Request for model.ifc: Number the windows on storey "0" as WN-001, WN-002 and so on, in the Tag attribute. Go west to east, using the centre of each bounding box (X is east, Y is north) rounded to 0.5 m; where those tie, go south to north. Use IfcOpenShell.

First a look at what the model holds.

```python
import ifcopenshell
import ifcopenshell.util.element
import ifcopenshell.util.placement

model = ifcopenshell.open("model.ifc")
print(model.schema)
storey = next(s for s in model.by_type("IfcBuildingStorey") if s.Name == "0")
windows = [e for e in ifcopenshell.util.element.get_decomposition(storey) if e.is_a("IfcWindow")]
for e in sorted(windows, key=lambda e: e.id()):
    origin = ifcopenshell.util.placement.get_local_placement(e.ObjectPlacement)[:3, 3]
    print(e.id(), e.Tag, e.Name, origin.round(2) + 0.0, sep=" | ")
```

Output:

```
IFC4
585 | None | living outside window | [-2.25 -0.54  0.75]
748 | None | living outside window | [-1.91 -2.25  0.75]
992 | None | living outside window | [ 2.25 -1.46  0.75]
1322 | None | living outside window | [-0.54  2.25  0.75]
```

```python
import ifcopenshell
import ifcopenshell.geom
import ifcopenshell.util.element
import ifcopenshell.util.shape

model = ifcopenshell.open("model.ifc")
settings = ifcopenshell.geom.settings()
settings.set("use-world-coords", True)


def centre(element):
    shape = ifcopenshell.geom.create_shape(settings, element)
    return ifcopenshell.util.shape.get_bbox_centroid(shape.geometry)


storey = next(s for s in model.by_type("IfcBuildingStorey") if s.Name == "0")
windows = [e for e in ifcopenshell.util.element.get_decomposition(storey) if e.is_a("IfcWindow")]

# Insertion points can sit at a corner or the storey origin, so sort by the geometry (in metres).
centres = {e: centre(e) for e in windows}
windows.sort(key=lambda e: (round(centres[e][0] / 0.5), centres[e][1]))

for i, e in enumerate(windows, start=1):
    number = f"WN-0{i:02d}"
    e.Tag = number
    print(e.id(), number)

model.write("model-out.ifc")
```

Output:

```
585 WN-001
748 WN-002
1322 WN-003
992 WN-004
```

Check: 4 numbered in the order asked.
